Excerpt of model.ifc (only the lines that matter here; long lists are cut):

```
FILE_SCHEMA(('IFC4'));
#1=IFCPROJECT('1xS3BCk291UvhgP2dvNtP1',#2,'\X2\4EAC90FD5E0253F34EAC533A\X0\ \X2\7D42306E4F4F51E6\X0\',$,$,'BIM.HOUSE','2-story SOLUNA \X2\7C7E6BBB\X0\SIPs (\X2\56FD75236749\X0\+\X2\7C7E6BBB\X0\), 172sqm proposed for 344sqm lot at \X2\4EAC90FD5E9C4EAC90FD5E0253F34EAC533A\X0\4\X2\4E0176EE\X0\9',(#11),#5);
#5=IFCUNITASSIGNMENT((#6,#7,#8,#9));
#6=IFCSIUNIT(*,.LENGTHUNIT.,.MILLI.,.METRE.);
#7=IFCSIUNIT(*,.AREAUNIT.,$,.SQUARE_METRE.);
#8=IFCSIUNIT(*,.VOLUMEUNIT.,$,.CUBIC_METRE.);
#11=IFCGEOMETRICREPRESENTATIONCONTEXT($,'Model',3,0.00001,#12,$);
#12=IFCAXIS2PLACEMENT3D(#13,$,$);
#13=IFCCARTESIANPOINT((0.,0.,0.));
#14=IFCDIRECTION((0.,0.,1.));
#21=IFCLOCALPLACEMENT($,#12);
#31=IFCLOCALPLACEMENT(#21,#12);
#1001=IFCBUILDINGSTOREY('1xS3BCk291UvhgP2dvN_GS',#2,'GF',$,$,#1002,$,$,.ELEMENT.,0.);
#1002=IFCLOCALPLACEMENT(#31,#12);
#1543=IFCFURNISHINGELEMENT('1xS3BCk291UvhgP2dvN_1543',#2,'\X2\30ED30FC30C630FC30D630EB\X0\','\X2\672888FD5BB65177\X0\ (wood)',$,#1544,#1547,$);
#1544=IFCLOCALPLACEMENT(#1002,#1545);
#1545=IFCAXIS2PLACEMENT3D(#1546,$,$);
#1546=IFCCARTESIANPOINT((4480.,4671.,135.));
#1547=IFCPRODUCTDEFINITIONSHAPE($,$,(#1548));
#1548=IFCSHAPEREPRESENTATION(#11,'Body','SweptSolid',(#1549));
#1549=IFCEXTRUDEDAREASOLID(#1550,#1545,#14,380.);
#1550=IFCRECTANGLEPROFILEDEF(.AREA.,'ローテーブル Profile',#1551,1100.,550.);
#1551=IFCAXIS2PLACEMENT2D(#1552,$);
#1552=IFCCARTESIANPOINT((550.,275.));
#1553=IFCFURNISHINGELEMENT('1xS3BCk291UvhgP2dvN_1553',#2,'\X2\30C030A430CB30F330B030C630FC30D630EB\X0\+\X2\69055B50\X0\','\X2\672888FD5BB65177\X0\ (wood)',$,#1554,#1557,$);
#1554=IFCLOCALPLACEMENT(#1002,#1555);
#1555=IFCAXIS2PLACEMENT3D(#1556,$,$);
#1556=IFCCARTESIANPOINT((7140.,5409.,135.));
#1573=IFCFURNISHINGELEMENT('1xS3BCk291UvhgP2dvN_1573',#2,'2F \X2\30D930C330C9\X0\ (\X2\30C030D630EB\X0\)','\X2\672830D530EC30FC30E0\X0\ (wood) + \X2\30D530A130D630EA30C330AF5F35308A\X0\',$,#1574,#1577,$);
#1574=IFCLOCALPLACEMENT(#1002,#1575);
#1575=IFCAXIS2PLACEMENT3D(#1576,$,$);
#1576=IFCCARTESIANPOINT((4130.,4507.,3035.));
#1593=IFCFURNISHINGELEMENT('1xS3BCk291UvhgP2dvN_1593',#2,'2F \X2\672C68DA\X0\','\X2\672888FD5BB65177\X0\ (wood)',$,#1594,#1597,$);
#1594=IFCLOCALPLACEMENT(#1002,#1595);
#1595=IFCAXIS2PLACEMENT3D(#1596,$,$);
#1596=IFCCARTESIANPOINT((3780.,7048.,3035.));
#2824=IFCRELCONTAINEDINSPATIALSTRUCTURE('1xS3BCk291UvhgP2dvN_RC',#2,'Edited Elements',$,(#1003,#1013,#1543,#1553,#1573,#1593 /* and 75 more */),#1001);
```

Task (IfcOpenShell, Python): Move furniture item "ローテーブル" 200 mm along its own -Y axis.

```python
import ifcopenshell
import ifcopenshell.api.geometry
import ifcopenshell.util.placement

model = ifcopenshell.open("model.ifc")

item = model.by_guid("1xS3BCk291UvhgP2dvN_1543")
matrix = ifcopenshell.util.placement.get_local_placement(item.ObjectPlacement)
matrix[:3, 3] -= matrix[:3, 1] * 200.0
ifcopenshell.api.geometry.edit_object_placement(model, product=item, matrix=matrix, is_si=False)

print(ifcopenshell.util.placement.get_local_placement(item.ObjectPlacement).round(3) + 0.0)

model.write("model-out.ifc")
```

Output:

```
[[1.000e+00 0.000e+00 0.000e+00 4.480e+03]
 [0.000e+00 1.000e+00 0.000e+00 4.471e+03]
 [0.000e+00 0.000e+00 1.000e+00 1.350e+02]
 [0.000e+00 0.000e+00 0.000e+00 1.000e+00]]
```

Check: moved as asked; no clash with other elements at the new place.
